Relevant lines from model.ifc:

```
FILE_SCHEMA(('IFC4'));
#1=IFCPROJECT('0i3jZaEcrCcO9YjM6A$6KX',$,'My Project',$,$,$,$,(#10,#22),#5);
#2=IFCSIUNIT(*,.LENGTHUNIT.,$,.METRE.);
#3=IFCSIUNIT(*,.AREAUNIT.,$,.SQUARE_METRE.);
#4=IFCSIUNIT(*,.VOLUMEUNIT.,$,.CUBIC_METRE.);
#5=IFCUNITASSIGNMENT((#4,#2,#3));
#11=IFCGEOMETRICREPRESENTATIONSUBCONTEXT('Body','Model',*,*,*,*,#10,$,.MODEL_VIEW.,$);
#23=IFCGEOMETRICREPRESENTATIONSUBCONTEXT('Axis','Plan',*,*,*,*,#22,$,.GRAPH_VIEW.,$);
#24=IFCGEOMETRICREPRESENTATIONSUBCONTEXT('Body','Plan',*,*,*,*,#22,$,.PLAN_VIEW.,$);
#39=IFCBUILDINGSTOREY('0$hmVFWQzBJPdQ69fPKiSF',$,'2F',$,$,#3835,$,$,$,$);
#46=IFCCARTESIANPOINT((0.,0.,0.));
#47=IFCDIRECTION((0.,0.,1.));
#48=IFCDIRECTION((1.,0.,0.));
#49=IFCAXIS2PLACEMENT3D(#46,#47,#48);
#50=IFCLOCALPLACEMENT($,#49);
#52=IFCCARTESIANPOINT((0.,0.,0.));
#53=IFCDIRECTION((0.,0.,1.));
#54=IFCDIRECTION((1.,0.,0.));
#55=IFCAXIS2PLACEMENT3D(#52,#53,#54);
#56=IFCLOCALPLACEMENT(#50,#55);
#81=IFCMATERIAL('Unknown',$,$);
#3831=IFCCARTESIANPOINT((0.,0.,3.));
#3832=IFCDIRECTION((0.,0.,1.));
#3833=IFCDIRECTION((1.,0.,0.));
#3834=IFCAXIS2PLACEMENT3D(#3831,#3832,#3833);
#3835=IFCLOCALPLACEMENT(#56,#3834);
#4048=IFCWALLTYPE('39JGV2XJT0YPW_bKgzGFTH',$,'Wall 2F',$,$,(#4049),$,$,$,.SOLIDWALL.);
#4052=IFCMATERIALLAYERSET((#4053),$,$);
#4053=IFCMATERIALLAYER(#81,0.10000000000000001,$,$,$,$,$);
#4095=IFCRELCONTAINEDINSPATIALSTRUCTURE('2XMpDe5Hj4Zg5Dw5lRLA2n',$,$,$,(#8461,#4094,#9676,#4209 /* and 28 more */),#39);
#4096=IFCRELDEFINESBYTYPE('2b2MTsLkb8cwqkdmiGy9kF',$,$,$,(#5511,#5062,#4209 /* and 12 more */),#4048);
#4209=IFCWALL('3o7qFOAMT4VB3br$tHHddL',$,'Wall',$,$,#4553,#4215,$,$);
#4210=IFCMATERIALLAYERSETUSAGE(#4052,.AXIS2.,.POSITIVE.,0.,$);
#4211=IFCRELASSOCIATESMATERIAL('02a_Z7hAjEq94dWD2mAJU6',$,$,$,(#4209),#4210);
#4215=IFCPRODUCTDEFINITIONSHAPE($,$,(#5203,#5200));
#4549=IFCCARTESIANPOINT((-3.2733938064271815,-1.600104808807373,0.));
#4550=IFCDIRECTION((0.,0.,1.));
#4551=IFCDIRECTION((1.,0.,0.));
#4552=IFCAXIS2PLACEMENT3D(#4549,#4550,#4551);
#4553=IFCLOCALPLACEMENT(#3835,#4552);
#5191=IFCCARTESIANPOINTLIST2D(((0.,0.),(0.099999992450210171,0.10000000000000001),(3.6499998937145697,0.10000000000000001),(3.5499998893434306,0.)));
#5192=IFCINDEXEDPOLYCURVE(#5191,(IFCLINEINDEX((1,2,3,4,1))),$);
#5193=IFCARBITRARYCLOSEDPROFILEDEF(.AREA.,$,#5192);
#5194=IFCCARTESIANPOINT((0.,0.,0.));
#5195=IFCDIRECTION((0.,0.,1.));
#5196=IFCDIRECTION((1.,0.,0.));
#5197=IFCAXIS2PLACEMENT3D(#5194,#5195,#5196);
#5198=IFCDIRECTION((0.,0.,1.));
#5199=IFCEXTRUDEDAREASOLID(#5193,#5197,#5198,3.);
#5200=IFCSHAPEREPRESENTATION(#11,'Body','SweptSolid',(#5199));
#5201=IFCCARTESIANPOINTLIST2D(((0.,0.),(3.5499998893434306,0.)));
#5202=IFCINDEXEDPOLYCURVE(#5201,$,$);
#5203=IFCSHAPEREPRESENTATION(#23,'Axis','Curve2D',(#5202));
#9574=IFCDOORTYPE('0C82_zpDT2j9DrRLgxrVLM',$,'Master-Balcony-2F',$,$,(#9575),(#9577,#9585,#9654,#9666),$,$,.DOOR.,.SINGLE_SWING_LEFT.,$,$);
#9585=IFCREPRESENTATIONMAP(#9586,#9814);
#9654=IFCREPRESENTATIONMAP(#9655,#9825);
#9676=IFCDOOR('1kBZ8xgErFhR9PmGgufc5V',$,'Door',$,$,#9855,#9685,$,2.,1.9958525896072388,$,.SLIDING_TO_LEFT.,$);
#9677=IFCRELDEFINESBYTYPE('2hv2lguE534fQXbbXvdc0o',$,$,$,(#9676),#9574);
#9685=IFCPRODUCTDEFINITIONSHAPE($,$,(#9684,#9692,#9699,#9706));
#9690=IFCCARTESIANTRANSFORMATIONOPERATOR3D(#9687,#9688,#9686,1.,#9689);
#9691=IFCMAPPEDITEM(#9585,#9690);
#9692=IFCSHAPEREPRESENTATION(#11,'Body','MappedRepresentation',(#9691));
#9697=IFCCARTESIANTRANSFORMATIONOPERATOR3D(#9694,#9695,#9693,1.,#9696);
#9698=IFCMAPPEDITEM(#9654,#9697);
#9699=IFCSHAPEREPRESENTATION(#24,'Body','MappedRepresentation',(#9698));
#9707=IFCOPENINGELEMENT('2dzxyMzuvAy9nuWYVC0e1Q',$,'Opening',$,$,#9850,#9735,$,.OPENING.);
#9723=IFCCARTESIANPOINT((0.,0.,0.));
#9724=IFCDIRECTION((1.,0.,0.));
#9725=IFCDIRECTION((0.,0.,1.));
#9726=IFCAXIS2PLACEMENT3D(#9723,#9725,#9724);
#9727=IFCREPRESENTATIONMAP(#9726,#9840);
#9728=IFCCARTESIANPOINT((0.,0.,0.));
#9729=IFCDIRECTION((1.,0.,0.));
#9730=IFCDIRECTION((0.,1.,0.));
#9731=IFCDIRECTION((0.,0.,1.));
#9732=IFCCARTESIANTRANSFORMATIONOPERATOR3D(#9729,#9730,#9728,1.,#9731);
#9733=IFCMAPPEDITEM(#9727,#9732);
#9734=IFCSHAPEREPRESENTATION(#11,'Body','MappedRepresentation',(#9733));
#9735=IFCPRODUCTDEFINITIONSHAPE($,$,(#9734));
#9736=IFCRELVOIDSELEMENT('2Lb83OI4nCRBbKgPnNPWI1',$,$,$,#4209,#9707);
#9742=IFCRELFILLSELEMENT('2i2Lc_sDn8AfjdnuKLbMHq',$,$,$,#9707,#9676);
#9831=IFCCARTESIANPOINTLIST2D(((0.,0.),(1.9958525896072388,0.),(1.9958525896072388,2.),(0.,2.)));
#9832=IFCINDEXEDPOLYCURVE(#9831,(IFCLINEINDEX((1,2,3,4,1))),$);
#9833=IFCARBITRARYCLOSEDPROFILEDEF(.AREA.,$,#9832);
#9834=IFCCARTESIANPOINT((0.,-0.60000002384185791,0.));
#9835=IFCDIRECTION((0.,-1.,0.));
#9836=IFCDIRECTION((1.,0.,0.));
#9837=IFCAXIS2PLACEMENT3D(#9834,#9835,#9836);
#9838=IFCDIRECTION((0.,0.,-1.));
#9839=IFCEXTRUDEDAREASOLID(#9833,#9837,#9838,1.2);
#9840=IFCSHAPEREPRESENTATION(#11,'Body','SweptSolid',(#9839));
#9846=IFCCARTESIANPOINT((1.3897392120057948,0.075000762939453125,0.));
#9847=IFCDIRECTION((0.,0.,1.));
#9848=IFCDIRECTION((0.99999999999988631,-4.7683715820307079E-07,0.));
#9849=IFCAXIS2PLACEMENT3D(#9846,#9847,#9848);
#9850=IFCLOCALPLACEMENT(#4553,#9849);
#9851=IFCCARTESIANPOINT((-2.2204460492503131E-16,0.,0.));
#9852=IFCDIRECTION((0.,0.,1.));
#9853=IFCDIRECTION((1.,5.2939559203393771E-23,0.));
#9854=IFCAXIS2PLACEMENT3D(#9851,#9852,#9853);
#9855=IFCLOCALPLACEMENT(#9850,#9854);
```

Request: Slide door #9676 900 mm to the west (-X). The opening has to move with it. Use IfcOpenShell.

```python
import ifcopenshell
import ifcopenshell.api.geometry
import ifcopenshell.util.placement

model = ifcopenshell.open("model.ifc")

door = model.by_guid("1kBZ8xgErFhR9PmGgufc5V")
opening = door.FillsVoids[0].RelatingOpeningElement
wall = opening.VoidsElements[0].RelatingBuildingElement

wall_matrix = ifcopenshell.util.placement.get_local_placement(wall.ObjectPlacement)
shift = wall_matrix[:3, 0] * -0.9
before = ifcopenshell.util.placement.get_local_placement(door.ObjectPlacement)[:3, 3].copy()

# The door is placed relative to its opening, so it follows when the opening moves.
matrix = ifcopenshell.util.placement.get_local_placement(opening.ObjectPlacement)
matrix[:3, 3] += shift
ifcopenshell.api.geometry.edit_object_placement(
    model, product=opening, matrix=matrix, is_si=False, should_transform_children=True
)

after = ifcopenshell.util.placement.get_local_placement(door.ObjectPlacement)[:3, 3]
print("door moved by", (after - before).round(3) + 0.0)

model.write("model-out.ifc")
```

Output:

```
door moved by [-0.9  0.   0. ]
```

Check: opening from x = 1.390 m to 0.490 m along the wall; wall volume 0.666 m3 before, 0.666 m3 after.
